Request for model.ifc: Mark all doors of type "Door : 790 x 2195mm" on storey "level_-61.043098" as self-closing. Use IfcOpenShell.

First a look at what the model holds.

```python
import ifcopenshell
import ifcopenshell.util.element

model = ifcopenshell.open("model.ifc")
print(model.schema)
storey = next(s for s in model.by_type("IfcBuildingStorey") if s.Name == "level_-61.043098")
doors = [e for e in ifcopenshell.util.element.get_decomposition(storey) if e.is_a("IfcDoor")]
seen = {}
for e in doors:
    element_type = ifcopenshell.util.element.get_type(e)
    key = (element_type.Name if element_type != e and element_type else None, ifcopenshell.util.element.get_pset(e, "Pset_DoorCommon", "SelfClosing"))
    seen[key] = seen.get(key, 0) + 1
for (name, value), count in sorted(seen.items(), key=str):
    print(count, "x", name, "|", value)
```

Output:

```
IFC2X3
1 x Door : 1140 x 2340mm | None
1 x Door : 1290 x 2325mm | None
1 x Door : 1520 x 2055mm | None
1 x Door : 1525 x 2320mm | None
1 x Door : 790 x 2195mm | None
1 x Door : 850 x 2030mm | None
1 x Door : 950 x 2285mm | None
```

```python
import ifcopenshell
import ifcopenshell.api.pset
import ifcopenshell.util.element

model = ifcopenshell.open("model.ifc")

storey = next(s for s in model.by_type("IfcBuildingStorey") if s.Name == "level_-61.043098")
doors = [e for e in ifcopenshell.util.element.get_decomposition(storey) if e.is_a("IfcDoor")]

count = 0
for e in doors:
    element_type = ifcopenshell.util.element.get_type(e)
    if element_type in (None, e) or element_type.Name != "Door : 790 x 2195mm":
        continue
    # add_pset returns the element's existing set when there is one.
    pset = ifcopenshell.api.pset.add_pset(model, product=e, name="Pset_DoorCommon")
    ifcopenshell.api.pset.edit_pset(model, pset=pset, properties={"SelfClosing": True})
    count += 1

print(count, "doors updated")

model.write("model_updated.ifc")
```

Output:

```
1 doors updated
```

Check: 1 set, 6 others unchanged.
